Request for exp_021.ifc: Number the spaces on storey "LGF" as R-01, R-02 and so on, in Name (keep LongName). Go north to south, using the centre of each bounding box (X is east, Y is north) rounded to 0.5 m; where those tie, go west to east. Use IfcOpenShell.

First a look at what the model holds.

```python
import ifcopenshell
import ifcopenshell.util.element
import ifcopenshell.util.placement

model = ifcopenshell.open("exp_021.ifc")
print(model.schema)
storey = next(s for s in model.by_type("IfcBuildingStorey") if s.Name == "LGF")
spaces = [e for e in ifcopenshell.util.element.get_decomposition(storey) if e.is_a("IfcSpace")]
for e in sorted(spaces, key=lambda e: e.id()):
    origin = ifcopenshell.util.placement.get_local_placement(e.ObjectPlacement)[:3, 3]
    print(e.id(), e.Name, e.LongName, origin.round(2) + 0.0, sep=" | ")
```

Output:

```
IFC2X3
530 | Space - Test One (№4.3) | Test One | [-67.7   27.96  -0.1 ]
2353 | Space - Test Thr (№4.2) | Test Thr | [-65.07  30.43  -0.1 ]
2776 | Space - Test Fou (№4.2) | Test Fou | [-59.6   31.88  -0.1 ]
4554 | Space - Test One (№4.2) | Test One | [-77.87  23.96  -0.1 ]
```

```python
import ifcopenshell
import ifcopenshell.geom
import ifcopenshell.util.element
import ifcopenshell.util.shape

model = ifcopenshell.open("exp_021.ifc")
settings = ifcopenshell.geom.settings()
settings.set("use-world-coords", True)


def centre(element):
    shape = ifcopenshell.geom.create_shape(settings, element)
    return ifcopenshell.util.shape.get_bbox_centroid(shape.geometry)


storey = next(s for s in model.by_type("IfcBuildingStorey") if s.Name == "LGF")
spaces = [e for e in ifcopenshell.util.element.get_decomposition(storey) if e.is_a("IfcSpace")]

# Insertion points can sit at a corner or the storey origin, so sort by the geometry (in metres).
centres = {e: centre(e) for e in spaces}
spaces.sort(key=lambda e: (-round(centres[e][1] / 0.5), centres[e][0]))

for i, e in enumerate(spaces, start=1):
    number = f"R-{i:02d}"
    e.Name = number
    print(e.id(), number)

model.write("exp_021_rev.ifc")
```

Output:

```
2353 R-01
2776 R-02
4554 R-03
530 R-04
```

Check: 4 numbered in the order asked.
